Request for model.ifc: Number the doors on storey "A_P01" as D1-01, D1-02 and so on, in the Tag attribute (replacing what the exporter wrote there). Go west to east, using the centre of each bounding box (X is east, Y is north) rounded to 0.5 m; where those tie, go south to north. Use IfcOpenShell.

First a look at what the model holds.

```python
import ifcopenshell
import ifcopenshell.util.element
import ifcopenshell.util.placement

model = ifcopenshell.open("model.ifc")
print(model.schema)
storey = next(s for s in model.by_type("IfcBuildingStorey") if s.Name == "A_P01")
doors = [e for e in ifcopenshell.util.element.get_decomposition(storey) if e.is_a("IfcDoor")]
for e in sorted(doors, key=lambda e: e.id()):
    origin = ifcopenshell.util.placement.get_local_placement(e.ObjectPlacement)[:3, 3]
    print(e.id(), e.Tag, e.Name, origin.round(2) + 0.0, sep=" | ")
```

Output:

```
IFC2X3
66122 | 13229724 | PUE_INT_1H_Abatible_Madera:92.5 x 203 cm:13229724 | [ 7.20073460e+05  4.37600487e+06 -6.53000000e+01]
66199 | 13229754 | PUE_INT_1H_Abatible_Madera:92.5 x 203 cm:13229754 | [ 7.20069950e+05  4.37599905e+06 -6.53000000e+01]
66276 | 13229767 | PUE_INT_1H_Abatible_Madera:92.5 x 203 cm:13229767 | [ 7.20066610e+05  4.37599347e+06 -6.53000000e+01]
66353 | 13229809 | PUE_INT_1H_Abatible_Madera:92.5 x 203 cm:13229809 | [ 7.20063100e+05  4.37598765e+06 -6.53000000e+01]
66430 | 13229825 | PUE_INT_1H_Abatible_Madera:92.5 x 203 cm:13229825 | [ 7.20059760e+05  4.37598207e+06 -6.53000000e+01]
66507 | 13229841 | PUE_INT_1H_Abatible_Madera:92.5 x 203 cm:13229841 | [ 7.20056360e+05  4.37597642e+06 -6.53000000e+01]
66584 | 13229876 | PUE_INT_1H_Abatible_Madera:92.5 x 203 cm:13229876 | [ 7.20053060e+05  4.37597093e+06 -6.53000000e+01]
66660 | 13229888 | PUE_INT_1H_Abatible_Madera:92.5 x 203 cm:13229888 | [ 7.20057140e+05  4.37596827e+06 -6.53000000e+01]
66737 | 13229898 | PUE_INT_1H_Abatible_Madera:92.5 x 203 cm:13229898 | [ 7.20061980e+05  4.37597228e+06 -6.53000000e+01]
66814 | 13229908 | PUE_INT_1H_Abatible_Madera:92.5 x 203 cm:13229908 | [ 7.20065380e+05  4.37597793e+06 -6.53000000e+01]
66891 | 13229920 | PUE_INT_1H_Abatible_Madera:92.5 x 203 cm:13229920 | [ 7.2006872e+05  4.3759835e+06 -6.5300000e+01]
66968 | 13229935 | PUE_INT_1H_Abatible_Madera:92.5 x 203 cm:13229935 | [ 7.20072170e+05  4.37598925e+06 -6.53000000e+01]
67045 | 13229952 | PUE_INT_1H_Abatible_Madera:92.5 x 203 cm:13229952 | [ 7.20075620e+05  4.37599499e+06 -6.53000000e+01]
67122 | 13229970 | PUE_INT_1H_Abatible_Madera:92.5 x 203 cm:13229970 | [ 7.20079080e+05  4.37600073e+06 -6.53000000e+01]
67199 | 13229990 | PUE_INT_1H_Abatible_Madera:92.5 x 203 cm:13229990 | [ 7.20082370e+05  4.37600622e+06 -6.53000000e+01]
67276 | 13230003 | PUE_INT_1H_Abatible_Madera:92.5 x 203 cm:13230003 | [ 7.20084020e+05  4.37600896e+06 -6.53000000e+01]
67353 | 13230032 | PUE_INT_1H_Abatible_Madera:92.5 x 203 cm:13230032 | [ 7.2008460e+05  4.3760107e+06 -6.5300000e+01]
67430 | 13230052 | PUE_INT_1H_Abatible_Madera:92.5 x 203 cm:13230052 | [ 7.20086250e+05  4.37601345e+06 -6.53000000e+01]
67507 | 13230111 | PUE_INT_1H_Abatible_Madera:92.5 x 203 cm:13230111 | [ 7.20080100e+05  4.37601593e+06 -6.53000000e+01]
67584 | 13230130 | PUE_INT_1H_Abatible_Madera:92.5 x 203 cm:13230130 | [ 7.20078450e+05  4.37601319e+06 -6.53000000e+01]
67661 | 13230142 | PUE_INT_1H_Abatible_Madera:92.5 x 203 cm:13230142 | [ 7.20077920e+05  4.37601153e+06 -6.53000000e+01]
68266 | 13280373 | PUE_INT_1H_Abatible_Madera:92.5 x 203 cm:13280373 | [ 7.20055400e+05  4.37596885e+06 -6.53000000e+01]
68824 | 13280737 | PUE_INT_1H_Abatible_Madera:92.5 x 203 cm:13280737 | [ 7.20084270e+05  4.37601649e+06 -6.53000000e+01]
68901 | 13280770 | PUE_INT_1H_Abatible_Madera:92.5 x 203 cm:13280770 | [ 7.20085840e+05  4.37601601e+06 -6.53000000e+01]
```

```python
import ifcopenshell
import ifcopenshell.geom
import ifcopenshell.util.element
import ifcopenshell.util.shape

model = ifcopenshell.open("model.ifc")
settings = ifcopenshell.geom.settings()
settings.set("use-world-coords", True)


def centre(element):
    shape = ifcopenshell.geom.create_shape(settings, element)
    return ifcopenshell.util.shape.get_bbox_centroid(shape.geometry)


storey = next(s for s in model.by_type("IfcBuildingStorey") if s.Name == "A_P01")
doors = [e for e in ifcopenshell.util.element.get_decomposition(storey) if e.is_a("IfcDoor")]

# Insertion points can sit at a corner or the storey origin, so sort by the geometry (in metres).
centres = {e: centre(e) for e in doors}
doors.sort(key=lambda e: (round(centres[e][0] / 0.5), centres[e][1]))

for i, e in enumerate(doors, start=1):
    number = f"D1-{i:02d}"
    e.Tag = number
    print(e.id(), number)

model.write("model_v2.ifc")
```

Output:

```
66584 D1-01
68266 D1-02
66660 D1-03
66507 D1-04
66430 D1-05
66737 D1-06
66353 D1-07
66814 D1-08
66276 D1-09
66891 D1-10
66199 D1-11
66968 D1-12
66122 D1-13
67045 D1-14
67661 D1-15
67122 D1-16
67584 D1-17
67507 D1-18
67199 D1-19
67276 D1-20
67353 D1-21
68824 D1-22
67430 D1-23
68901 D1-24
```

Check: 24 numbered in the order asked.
